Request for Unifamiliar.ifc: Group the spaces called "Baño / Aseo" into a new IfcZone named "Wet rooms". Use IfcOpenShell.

First a look at what the model holds.

```python
import ifcopenshell

model = ifcopenshell.open("Unifamiliar.ifc")
print(model.schema)
seen = {}
for space in model.by_type("IfcSpace"):
    seen[space.LongName] = seen.get(space.LongName, 0) + 1
for name, count in sorted(seen.items(), key=str):
    print(count, "x", name)
print("zones:", [z.Name for z in model.by_type("IfcZone")][:20])
```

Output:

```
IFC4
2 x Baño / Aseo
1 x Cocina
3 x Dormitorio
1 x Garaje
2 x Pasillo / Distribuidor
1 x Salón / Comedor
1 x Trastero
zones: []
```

```python
import ifcopenshell
import ifcopenshell.api.group
import ifcopenshell.api.root

model = ifcopenshell.open("Unifamiliar.ifc")

names = {"Baño / Aseo"}
spaces = [s for s in model.by_type("IfcSpace") if s.LongName in names]

zone = ifcopenshell.api.root.create_entity(model, ifc_class="IfcZone", name="Wet rooms")
ifcopenshell.api.group.assign_group(model, products=spaces, group=zone)
print(len(spaces), "spaces in", zone.Name)

model.write("Unifamiliar-out.ifc")
```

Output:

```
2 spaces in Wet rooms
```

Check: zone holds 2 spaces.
